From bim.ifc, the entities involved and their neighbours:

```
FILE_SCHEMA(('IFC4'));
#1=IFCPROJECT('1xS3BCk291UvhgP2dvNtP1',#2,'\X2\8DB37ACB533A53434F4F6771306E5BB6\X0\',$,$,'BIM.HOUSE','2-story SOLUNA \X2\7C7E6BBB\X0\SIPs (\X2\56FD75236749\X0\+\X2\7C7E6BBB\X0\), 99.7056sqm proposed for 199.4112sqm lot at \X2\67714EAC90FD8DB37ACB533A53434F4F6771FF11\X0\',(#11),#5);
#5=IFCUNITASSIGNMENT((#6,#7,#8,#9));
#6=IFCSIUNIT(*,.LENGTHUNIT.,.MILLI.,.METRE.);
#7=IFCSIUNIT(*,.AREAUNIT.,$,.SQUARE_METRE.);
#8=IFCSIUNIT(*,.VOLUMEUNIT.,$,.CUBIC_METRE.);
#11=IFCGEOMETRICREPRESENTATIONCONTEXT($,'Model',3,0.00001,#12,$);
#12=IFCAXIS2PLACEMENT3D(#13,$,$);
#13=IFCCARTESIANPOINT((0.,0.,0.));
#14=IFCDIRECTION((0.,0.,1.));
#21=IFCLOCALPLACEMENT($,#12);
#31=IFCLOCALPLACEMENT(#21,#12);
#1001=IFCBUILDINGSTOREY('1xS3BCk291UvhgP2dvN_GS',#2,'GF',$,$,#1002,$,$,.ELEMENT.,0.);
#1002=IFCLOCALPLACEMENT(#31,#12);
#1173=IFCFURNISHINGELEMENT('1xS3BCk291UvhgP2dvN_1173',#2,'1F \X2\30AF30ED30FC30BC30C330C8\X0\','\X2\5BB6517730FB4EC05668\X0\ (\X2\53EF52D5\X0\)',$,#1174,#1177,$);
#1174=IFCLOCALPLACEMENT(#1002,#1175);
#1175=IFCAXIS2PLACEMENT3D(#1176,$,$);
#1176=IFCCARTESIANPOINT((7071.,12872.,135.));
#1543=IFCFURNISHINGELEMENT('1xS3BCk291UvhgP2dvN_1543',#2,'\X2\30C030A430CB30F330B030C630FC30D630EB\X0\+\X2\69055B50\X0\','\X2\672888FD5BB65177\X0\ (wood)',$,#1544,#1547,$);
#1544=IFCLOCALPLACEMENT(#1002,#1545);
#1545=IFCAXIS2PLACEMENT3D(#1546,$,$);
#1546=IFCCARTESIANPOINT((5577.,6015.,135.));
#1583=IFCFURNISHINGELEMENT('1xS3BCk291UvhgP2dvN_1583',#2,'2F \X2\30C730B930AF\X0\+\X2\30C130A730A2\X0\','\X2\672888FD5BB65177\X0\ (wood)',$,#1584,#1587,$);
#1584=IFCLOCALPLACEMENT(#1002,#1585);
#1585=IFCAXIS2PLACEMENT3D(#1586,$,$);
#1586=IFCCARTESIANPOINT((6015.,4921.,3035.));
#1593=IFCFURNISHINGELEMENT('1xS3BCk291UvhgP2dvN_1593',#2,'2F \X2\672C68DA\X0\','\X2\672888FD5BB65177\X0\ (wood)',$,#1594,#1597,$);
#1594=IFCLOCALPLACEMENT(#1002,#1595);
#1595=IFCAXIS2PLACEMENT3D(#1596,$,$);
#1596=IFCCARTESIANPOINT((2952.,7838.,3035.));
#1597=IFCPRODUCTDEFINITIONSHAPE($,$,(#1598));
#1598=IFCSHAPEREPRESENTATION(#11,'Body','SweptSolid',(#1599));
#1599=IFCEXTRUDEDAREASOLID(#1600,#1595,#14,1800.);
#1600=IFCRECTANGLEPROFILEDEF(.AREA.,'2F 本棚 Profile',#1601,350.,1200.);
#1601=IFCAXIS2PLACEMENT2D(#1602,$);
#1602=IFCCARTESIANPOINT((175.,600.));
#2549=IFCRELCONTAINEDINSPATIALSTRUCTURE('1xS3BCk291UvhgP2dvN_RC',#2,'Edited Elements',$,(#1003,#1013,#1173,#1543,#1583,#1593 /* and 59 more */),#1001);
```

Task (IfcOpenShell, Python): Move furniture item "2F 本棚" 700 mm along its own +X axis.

```python
import ifcopenshell
import ifcopenshell.api.geometry
import ifcopenshell.util.placement

model = ifcopenshell.open("bim.ifc")

item = model.by_id(1593)
matrix = ifcopenshell.util.placement.get_local_placement(item.ObjectPlacement)
matrix[:3, 3] += matrix[:3, 0] * 700.0
ifcopenshell.api.geometry.edit_object_placement(model, product=item, matrix=matrix, is_si=False)

print(ifcopenshell.util.placement.get_local_placement(item.ObjectPlacement).round(3) + 0.0)

model.write("bim_updated.ifc")
```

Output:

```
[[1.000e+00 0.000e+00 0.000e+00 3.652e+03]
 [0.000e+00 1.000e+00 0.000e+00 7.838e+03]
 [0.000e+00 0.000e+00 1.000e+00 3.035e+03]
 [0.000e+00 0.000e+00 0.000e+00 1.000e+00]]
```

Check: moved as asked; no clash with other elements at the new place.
